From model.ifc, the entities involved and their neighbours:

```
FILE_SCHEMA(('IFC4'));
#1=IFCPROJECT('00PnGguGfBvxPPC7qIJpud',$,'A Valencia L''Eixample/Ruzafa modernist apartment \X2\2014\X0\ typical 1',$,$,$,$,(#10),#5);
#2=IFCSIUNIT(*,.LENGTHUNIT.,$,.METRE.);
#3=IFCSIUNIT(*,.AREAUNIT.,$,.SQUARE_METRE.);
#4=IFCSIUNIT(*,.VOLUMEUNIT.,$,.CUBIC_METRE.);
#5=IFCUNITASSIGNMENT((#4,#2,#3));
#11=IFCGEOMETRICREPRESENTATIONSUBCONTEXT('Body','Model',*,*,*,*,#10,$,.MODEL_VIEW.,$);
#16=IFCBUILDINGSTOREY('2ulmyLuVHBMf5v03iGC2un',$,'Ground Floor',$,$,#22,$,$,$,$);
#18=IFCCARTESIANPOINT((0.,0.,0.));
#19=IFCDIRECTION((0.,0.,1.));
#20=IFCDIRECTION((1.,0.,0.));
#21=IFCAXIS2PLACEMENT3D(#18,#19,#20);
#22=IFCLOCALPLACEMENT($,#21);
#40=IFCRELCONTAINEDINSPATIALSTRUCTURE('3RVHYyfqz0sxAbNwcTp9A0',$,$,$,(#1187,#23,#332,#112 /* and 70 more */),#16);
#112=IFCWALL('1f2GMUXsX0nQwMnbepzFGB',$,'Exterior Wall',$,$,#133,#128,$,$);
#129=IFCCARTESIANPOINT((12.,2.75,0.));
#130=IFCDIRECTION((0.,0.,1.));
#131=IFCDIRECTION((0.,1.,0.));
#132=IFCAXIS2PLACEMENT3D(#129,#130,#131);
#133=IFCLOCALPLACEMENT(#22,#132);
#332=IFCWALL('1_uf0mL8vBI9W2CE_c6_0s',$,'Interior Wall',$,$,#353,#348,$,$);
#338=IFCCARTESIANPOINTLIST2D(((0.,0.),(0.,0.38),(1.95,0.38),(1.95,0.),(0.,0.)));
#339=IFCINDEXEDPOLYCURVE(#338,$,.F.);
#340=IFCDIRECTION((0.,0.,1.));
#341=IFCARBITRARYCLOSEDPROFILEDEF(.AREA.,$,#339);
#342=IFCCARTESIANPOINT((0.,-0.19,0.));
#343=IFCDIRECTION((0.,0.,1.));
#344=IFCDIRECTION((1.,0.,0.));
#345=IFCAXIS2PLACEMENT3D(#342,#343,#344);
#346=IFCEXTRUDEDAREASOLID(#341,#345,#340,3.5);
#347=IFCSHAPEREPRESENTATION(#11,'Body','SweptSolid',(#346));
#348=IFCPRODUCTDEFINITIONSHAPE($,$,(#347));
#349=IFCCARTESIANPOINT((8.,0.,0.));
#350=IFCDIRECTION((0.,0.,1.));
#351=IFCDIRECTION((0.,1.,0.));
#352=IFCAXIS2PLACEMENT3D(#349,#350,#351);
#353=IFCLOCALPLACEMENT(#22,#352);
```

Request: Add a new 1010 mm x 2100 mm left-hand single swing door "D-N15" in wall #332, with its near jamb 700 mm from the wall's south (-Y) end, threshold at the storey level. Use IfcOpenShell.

```python
import numpy as np
import ifcopenshell
import ifcopenshell.api.feature
import ifcopenshell.api.geometry
import ifcopenshell.api.root
import ifcopenshell.api.spatial
import ifcopenshell.geom
import ifcopenshell.util.element
import ifcopenshell.util.placement
import ifcopenshell.util.representation
import ifcopenshell.util.shape
import ifcopenshell.util.unit

model = ifcopenshell.open("model.ifc")
unit_scale = ifcopenshell.util.unit.calculate_unit_scale(model)
settings = ifcopenshell.geom.settings()


def volume(element):
    """Net volume in cubic metres, openings subtracted."""
    shape = ifcopenshell.geom.create_shape(settings, element)
    return ifcopenshell.util.shape.get_volume(shape.geometry)


wall = model.by_id(332)
storey = ifcopenshell.util.element.get_container(wall, ifc_class="IfcBuildingStorey")
context = ifcopenshell.util.representation.get_context(model, "Model", "Body", "MODEL_VIEW")
before = volume(wall)

width, height, from_end, sill = 1.01, 2.1, 0.7, 0.0  # metres

# The wall runs along its own X axis, and the end named is its -X end.
wall_shape = ifcopenshell.geom.create_shape(settings, wall)
x, y, z = ifcopenshell.util.shape.get_vertices(wall_shape.geometry).T
start = x.min() + from_end
face, thickness = float(y.min()), float(y.max() - y.min())
wall_matrix = ifcopenshell.util.placement.get_local_placement(wall.ObjectPlacement)
level = ifcopenshell.util.placement.get_local_placement(storey.ObjectPlacement)[2, 3]


def in_wall(x, y):
    """Placement at x, y metres in the wall's axes, at sill height."""
    matrix = wall_matrix.copy()
    matrix[:, 3] = wall_matrix @ np.array([x / unit_scale, y / unit_scale, 0.0, 1.0])
    matrix[2, 3] = level + sill / unit_scale
    return matrix


# Opening: a box that overshoots both wall faces by 50 mm.
opening = ifcopenshell.api.root.create_entity(model, ifc_class="IfcOpeningElement", predefined_type="OPENING")
box = ifcopenshell.api.geometry.add_wall_representation(
    model, context=context, length=width, height=height, thickness=thickness + 0.1
)
ifcopenshell.api.geometry.assign_representation(model, product=opening, representation=box)
ifcopenshell.api.geometry.edit_object_placement(model, product=opening, matrix=in_wall(start, face - 0.05), is_si=False)
ifcopenshell.api.feature.add_feature(model, feature=opening, element=wall)

door = ifcopenshell.api.root.create_entity(model, ifc_class="IfcDoor", name="D-N15", predefined_type="DOOR")
door.OverallWidth, door.OverallHeight = width / unit_scale, height / unit_scale
door.OperationType = "SINGLE_SWING_LEFT"
body = ifcopenshell.api.geometry.add_door_representation(
    model,
    context=context,
    overall_width=door.OverallWidth,
    overall_height=door.OverallHeight,
    operation_type="SINGLE_SWING_LEFT",
    lining_properties={"LiningDepth": thickness / unit_scale, "ThresholdDepth": thickness / unit_scale},
)
ifcopenshell.api.geometry.assign_representation(model, product=door, representation=body)
ifcopenshell.api.spatial.assign_container(model, products=[door], relating_structure=storey)
ifcopenshell.api.feature.add_filling(model, opening=opening, element=door)

# The lining spans the wall, so the door starts at the wall face.
ifcopenshell.api.geometry.edit_object_placement(model, product=door, matrix=in_wall(start, face), is_si=False)

after = volume(wall)

print(f"wall volume {before:.3f} -> {after:.3f} m3")

model.write("model-out.ifc")
```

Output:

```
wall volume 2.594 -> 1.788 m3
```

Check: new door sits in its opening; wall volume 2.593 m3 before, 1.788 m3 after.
